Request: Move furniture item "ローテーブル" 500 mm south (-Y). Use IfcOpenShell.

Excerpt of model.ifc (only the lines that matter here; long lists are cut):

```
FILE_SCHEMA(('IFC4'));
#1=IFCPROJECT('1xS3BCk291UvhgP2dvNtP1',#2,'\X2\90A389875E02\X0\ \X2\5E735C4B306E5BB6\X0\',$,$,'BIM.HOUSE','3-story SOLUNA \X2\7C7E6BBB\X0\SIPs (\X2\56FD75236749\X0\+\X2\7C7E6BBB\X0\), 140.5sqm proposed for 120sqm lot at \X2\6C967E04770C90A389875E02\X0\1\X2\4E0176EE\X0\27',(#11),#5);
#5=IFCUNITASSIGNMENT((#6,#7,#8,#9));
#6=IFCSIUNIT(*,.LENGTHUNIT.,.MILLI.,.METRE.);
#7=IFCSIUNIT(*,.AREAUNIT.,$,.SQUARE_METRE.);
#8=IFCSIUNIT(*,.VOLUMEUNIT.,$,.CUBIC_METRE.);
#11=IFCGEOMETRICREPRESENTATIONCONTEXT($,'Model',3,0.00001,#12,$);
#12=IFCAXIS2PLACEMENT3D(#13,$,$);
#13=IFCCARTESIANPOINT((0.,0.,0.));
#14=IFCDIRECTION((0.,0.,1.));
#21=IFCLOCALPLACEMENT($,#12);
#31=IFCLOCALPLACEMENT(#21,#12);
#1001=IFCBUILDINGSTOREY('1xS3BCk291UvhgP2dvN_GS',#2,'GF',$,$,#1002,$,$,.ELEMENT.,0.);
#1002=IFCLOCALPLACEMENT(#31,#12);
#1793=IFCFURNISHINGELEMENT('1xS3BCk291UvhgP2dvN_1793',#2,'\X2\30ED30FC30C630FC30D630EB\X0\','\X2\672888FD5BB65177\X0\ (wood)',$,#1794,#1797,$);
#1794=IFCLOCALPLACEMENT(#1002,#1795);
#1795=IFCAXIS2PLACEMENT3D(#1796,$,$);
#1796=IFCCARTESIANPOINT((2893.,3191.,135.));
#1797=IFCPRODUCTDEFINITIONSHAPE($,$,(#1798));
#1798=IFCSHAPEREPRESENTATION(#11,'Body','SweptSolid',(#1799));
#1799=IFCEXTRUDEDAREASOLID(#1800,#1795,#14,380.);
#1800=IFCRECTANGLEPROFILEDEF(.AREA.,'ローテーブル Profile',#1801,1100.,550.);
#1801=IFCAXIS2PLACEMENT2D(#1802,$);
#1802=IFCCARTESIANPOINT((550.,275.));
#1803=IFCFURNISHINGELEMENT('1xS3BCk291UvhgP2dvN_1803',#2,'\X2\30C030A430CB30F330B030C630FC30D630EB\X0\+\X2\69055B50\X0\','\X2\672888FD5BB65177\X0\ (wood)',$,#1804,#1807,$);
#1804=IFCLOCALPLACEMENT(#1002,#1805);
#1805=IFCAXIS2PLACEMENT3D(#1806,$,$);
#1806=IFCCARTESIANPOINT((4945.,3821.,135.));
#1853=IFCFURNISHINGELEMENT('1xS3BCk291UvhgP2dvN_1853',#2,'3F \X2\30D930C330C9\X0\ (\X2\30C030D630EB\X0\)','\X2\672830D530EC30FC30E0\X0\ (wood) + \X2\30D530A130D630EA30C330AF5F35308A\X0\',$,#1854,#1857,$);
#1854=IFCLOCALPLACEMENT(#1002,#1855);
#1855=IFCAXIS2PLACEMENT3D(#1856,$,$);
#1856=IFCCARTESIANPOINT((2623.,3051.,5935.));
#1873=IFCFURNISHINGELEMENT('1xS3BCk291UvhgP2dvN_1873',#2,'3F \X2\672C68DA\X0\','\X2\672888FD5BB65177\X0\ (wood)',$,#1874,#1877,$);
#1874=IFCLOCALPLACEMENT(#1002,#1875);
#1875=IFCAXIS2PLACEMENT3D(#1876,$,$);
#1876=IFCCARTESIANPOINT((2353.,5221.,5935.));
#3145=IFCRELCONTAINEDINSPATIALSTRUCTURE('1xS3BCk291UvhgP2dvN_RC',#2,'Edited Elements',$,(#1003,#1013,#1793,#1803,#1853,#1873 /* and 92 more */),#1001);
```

```python
import ifcopenshell
import ifcopenshell.api.geometry
import ifcopenshell.util.placement
import ifcopenshell.util.unit

model = ifcopenshell.open("model.ifc")
unit_scale = ifcopenshell.util.unit.calculate_unit_scale(model)

item = model.by_guid("1xS3BCk291UvhgP2dvN_1793")
matrix = ifcopenshell.util.placement.get_local_placement(item.ObjectPlacement)
matrix[1, 3] -= 0.5 / unit_scale
ifcopenshell.api.geometry.edit_object_placement(model, product=item, matrix=matrix, is_si=False)

print(ifcopenshell.util.placement.get_local_placement(item.ObjectPlacement).round(3) + 0.0)

model.write("model-out.ifc")
```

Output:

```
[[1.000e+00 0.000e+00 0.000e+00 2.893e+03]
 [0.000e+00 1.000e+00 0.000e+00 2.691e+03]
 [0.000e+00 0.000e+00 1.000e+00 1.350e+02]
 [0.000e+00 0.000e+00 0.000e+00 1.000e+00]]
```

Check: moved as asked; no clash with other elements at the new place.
